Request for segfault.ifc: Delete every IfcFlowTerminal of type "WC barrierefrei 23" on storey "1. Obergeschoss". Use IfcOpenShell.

First a look at what the model holds.

```python
import ifcopenshell
import ifcopenshell.util.element

model = ifcopenshell.open("segfault.ifc")
print(model.schema)
storey = next(s for s in model.by_type("IfcBuildingStorey") if s.Name == "1. Obergeschoss")
terminals = [e for e in ifcopenshell.util.element.get_decomposition(storey) if e.is_a("IfcFlowTerminal")]
seen = {}
for e in terminals:
    element_type = ifcopenshell.util.element.get_type(e)
    name = element_type.Name if element_type not in (None, e) else None
    seen[name] = seen.get(name, 0) + 1
for name, count in sorted(seen.items(), key=str):
    print(count, "x", name)
```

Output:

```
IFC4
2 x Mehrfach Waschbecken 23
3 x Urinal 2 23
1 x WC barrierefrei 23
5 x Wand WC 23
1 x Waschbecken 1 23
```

```python
import ifcopenshell
import ifcopenshell.api.root
import ifcopenshell.util.element

model = ifcopenshell.open("segfault.ifc")

storey = next(s for s in model.by_type("IfcBuildingStorey") if s.Name == "1. Obergeschoss")
terminals = [e for e in ifcopenshell.util.element.get_decomposition(storey) if e.is_a("IfcFlowTerminal")]
targets = [e for e in terminals if (t := ifcopenshell.util.element.get_type(e)) not in (None, e) and t.Name == "WC barrierefrei 23"]

for e in targets:
    ifcopenshell.api.root.remove_product(model, product=e)
print(len(targets), "removed")

model.write("segfault_updated.ifc")
```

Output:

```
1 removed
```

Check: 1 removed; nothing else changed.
